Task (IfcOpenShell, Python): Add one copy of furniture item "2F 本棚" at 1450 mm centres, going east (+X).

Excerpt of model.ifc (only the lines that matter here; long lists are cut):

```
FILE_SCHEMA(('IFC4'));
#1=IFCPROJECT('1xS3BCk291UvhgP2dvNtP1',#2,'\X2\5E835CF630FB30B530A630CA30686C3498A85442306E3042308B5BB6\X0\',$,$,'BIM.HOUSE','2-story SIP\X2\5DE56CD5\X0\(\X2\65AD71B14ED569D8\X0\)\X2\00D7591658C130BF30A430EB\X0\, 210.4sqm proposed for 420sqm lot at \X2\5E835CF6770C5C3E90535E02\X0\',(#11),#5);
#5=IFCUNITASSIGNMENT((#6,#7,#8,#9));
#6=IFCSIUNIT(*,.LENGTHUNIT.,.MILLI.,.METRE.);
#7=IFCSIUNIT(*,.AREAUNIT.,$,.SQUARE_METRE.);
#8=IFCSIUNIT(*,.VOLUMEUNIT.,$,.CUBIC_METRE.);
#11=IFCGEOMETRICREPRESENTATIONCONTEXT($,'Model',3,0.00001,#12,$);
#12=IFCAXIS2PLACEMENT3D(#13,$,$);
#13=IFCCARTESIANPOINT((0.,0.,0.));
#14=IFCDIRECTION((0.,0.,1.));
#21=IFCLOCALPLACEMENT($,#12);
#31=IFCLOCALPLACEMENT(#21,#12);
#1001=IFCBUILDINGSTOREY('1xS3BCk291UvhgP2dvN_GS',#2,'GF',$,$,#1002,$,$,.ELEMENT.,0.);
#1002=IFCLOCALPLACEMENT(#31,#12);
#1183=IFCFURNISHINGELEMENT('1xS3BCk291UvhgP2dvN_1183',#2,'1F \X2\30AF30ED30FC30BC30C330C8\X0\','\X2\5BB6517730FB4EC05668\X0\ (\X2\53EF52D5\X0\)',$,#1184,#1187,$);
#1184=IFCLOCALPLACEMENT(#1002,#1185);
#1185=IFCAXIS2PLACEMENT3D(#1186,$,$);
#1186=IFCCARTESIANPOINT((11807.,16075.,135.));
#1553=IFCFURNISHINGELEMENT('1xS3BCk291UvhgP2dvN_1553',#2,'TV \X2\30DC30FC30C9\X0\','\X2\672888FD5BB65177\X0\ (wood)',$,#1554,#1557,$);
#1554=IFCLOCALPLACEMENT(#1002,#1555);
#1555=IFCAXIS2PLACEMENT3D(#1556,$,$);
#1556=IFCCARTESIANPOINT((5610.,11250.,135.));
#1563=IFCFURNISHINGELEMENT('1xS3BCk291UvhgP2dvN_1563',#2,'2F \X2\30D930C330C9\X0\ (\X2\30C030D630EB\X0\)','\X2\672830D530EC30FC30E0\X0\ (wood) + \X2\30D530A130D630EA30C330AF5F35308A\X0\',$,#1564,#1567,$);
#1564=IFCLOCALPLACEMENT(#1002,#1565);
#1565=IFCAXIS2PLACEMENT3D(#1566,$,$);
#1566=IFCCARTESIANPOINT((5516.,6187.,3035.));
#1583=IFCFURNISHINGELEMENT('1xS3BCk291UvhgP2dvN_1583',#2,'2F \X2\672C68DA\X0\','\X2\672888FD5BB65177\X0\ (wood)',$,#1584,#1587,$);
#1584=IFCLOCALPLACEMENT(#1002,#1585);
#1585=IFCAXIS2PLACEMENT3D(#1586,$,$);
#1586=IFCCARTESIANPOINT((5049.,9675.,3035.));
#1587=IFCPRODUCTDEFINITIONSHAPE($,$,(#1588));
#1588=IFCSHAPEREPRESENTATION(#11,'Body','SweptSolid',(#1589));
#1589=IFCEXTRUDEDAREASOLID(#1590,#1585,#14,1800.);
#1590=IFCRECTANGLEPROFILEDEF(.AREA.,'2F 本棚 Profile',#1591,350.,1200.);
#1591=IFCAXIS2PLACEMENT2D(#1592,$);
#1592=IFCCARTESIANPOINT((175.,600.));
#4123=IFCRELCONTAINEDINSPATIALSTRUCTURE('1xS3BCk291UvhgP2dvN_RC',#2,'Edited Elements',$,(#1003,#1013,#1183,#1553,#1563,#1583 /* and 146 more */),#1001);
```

```python
import numpy as np
import ifcopenshell
import ifcopenshell.api.geometry
import ifcopenshell.api.root
import ifcopenshell.util.element
import ifcopenshell.util.placement
import ifcopenshell.util.unit

model = ifcopenshell.open("model.ifc")
unit_scale = ifcopenshell.util.unit.calculate_unit_scale(model)


def reuse_history(source, copy):
    """copy_class also copies each property set's owner history, people and application; keep the originals."""
    for rel in copy.IsDefinedBy:
        if rel.is_a("IfcRelDefinesByProperties") and (history := rel.RelatingPropertyDefinition.OwnerHistory):
            rel.RelatingPropertyDefinition.OwnerHistory = source.OwnerHistory
            ifcopenshell.util.element.remove_deep2(model, history)


source = model.by_id(1583)
base = ifcopenshell.util.placement.get_local_placement(source.ObjectPlacement)
step = np.array([1.0, 0.0, 0.0]) * 1.45 / unit_scale

for i in range(1, 2):
    copy = ifcopenshell.api.root.copy_class(model, product=source)
    copy.Representation = ifcopenshell.util.element.copy_deep(
        model, source.Representation, exclude=["IfcGeometricRepresentationContext", "IfcRepresentationMap"]
    )
    reuse_history(source, copy)
    matrix = base.copy()
    matrix[:3, 3] += i * step
    print("added at", matrix[:3, 3].round(3) + 0.0)
    ifcopenshell.api.geometry.edit_object_placement(model, product=copy, matrix=matrix, is_si=False)

model.write("model_rev.ifc")
```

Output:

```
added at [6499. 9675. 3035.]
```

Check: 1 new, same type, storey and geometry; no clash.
